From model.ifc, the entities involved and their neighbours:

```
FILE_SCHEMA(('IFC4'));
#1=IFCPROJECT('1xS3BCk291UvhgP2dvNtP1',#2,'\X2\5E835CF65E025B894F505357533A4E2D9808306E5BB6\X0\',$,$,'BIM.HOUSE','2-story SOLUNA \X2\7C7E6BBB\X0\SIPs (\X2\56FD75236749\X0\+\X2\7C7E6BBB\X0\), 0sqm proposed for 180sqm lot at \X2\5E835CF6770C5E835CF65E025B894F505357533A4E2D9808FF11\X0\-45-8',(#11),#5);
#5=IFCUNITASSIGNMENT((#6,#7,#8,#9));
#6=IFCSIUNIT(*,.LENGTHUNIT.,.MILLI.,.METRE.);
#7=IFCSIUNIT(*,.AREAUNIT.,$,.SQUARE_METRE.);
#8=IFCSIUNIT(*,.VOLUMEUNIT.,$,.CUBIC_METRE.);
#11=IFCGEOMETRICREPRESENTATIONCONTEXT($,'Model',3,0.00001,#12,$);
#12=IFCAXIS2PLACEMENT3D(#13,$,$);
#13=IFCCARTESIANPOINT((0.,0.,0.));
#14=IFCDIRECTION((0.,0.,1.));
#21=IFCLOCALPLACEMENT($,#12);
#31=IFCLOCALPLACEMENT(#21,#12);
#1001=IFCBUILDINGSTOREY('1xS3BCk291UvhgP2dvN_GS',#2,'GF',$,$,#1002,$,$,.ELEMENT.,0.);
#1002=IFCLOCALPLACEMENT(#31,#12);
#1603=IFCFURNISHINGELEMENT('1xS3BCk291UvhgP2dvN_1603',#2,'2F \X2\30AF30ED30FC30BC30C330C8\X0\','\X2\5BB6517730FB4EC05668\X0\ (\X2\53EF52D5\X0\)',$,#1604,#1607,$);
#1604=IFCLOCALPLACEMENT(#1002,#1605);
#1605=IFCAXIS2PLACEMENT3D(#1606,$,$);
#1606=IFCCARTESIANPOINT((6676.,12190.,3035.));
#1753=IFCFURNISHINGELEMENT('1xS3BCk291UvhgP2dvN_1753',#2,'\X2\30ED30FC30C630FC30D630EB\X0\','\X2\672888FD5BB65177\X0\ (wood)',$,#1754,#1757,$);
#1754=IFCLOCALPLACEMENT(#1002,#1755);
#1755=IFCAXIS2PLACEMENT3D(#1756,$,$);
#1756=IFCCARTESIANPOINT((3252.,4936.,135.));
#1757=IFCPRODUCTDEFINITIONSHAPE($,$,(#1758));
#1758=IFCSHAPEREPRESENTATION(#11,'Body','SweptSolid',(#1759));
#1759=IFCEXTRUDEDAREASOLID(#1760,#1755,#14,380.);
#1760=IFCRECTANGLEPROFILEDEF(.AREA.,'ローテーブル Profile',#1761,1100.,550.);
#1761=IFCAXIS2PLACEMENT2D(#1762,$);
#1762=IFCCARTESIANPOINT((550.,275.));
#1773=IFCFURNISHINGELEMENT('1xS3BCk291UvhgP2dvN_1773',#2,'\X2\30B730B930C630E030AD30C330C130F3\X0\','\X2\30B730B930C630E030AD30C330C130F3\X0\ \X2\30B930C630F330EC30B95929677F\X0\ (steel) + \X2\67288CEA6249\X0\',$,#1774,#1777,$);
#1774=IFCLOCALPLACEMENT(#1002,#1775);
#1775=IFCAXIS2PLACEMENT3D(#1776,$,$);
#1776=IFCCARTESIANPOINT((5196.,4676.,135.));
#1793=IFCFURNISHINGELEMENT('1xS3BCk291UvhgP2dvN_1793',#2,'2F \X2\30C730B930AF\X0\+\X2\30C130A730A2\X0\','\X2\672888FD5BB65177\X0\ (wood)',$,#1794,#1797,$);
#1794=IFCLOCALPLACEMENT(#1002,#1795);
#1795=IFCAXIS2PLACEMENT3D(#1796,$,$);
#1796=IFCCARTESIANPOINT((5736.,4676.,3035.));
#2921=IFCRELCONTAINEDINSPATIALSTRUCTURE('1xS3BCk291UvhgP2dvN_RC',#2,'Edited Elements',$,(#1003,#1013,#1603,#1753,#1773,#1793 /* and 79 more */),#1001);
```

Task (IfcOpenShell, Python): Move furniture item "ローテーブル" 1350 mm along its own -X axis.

```python
import ifcopenshell
import ifcopenshell.api.geometry
import ifcopenshell.util.placement

model = ifcopenshell.open("model.ifc")

item = model.by_guid("1xS3BCk291UvhgP2dvN_1753")
matrix = ifcopenshell.util.placement.get_local_placement(item.ObjectPlacement)
matrix[:3, 3] -= matrix[:3, 0] * 1350.0
ifcopenshell.api.geometry.edit_object_placement(model, product=item, matrix=matrix, is_si=False)

print(ifcopenshell.util.placement.get_local_placement(item.ObjectPlacement).round(3) + 0.0)

model.write("model_rev.ifc")
```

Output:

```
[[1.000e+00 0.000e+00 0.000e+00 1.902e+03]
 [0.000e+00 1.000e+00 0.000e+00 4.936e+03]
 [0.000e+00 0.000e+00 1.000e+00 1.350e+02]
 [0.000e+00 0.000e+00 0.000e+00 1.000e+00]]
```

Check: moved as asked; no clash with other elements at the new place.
